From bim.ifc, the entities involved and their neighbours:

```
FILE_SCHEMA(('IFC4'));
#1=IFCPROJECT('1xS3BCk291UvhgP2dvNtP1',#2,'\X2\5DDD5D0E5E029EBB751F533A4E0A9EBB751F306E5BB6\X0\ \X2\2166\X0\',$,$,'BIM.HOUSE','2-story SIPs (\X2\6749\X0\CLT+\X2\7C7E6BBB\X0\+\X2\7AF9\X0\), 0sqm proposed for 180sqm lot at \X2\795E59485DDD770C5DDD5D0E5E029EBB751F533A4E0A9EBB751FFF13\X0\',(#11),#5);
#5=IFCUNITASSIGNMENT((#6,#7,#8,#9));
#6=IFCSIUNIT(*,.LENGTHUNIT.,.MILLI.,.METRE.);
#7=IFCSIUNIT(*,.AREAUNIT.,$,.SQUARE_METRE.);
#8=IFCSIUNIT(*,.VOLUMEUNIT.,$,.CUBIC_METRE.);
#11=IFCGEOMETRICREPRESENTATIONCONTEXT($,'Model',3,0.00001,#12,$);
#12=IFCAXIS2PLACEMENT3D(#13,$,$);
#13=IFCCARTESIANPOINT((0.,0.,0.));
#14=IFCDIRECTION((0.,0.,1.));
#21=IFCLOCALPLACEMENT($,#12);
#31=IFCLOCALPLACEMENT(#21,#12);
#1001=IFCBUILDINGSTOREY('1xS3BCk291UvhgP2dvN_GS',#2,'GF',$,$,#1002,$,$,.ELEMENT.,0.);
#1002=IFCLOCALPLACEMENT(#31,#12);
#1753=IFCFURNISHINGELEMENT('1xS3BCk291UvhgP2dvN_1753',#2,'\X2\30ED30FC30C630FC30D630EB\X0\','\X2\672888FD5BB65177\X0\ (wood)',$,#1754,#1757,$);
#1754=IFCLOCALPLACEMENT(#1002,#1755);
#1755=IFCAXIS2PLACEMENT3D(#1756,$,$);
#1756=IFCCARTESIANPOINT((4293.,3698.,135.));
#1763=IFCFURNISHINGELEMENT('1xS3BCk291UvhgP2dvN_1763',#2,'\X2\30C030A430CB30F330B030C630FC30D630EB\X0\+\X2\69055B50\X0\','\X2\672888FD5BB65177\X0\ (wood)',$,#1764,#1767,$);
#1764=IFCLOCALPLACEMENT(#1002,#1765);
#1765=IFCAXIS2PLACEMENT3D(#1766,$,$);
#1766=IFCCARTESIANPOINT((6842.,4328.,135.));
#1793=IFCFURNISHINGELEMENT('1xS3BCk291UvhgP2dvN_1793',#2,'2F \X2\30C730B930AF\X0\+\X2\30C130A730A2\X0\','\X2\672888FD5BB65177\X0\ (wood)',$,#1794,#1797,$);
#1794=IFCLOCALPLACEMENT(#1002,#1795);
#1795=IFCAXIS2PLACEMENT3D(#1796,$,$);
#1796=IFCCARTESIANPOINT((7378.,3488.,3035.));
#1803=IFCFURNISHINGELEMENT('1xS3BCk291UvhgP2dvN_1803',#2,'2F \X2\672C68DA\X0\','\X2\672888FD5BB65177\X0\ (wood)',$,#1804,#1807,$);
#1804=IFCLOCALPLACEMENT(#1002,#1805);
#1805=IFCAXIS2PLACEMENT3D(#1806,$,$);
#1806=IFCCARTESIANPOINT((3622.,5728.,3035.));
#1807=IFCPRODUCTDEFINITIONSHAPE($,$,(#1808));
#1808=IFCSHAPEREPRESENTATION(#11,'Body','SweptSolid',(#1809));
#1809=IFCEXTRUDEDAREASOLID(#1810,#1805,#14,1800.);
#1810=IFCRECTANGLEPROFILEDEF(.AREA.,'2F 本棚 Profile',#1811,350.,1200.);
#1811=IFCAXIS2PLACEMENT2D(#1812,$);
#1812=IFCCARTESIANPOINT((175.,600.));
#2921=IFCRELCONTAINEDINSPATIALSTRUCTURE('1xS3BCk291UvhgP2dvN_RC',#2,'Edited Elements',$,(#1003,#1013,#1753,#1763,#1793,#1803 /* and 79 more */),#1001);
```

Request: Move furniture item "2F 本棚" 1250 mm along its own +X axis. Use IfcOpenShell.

```python
import ifcopenshell
import ifcopenshell.api.geometry
import ifcopenshell.util.placement
import ifcopenshell.util.unit

model = ifcopenshell.open("bim.ifc")
unit_scale = ifcopenshell.util.unit.calculate_unit_scale(model)

item = model.by_guid("1xS3BCk291UvhgP2dvN_1803")
matrix = ifcopenshell.util.placement.get_local_placement(item.ObjectPlacement)
matrix[:3, 3] += matrix[:3, 0] * 1.25 / unit_scale
ifcopenshell.api.geometry.edit_object_placement(model, product=item, matrix=matrix, is_si=False)

print(ifcopenshell.util.placement.get_local_placement(item.ObjectPlacement).round(3) + 0.0)

model.write("bim_v2.ifc")
```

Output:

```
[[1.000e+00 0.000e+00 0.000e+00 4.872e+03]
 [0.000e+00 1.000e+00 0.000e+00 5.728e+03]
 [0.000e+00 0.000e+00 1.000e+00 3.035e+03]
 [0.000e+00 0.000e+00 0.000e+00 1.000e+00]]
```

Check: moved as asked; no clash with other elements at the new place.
